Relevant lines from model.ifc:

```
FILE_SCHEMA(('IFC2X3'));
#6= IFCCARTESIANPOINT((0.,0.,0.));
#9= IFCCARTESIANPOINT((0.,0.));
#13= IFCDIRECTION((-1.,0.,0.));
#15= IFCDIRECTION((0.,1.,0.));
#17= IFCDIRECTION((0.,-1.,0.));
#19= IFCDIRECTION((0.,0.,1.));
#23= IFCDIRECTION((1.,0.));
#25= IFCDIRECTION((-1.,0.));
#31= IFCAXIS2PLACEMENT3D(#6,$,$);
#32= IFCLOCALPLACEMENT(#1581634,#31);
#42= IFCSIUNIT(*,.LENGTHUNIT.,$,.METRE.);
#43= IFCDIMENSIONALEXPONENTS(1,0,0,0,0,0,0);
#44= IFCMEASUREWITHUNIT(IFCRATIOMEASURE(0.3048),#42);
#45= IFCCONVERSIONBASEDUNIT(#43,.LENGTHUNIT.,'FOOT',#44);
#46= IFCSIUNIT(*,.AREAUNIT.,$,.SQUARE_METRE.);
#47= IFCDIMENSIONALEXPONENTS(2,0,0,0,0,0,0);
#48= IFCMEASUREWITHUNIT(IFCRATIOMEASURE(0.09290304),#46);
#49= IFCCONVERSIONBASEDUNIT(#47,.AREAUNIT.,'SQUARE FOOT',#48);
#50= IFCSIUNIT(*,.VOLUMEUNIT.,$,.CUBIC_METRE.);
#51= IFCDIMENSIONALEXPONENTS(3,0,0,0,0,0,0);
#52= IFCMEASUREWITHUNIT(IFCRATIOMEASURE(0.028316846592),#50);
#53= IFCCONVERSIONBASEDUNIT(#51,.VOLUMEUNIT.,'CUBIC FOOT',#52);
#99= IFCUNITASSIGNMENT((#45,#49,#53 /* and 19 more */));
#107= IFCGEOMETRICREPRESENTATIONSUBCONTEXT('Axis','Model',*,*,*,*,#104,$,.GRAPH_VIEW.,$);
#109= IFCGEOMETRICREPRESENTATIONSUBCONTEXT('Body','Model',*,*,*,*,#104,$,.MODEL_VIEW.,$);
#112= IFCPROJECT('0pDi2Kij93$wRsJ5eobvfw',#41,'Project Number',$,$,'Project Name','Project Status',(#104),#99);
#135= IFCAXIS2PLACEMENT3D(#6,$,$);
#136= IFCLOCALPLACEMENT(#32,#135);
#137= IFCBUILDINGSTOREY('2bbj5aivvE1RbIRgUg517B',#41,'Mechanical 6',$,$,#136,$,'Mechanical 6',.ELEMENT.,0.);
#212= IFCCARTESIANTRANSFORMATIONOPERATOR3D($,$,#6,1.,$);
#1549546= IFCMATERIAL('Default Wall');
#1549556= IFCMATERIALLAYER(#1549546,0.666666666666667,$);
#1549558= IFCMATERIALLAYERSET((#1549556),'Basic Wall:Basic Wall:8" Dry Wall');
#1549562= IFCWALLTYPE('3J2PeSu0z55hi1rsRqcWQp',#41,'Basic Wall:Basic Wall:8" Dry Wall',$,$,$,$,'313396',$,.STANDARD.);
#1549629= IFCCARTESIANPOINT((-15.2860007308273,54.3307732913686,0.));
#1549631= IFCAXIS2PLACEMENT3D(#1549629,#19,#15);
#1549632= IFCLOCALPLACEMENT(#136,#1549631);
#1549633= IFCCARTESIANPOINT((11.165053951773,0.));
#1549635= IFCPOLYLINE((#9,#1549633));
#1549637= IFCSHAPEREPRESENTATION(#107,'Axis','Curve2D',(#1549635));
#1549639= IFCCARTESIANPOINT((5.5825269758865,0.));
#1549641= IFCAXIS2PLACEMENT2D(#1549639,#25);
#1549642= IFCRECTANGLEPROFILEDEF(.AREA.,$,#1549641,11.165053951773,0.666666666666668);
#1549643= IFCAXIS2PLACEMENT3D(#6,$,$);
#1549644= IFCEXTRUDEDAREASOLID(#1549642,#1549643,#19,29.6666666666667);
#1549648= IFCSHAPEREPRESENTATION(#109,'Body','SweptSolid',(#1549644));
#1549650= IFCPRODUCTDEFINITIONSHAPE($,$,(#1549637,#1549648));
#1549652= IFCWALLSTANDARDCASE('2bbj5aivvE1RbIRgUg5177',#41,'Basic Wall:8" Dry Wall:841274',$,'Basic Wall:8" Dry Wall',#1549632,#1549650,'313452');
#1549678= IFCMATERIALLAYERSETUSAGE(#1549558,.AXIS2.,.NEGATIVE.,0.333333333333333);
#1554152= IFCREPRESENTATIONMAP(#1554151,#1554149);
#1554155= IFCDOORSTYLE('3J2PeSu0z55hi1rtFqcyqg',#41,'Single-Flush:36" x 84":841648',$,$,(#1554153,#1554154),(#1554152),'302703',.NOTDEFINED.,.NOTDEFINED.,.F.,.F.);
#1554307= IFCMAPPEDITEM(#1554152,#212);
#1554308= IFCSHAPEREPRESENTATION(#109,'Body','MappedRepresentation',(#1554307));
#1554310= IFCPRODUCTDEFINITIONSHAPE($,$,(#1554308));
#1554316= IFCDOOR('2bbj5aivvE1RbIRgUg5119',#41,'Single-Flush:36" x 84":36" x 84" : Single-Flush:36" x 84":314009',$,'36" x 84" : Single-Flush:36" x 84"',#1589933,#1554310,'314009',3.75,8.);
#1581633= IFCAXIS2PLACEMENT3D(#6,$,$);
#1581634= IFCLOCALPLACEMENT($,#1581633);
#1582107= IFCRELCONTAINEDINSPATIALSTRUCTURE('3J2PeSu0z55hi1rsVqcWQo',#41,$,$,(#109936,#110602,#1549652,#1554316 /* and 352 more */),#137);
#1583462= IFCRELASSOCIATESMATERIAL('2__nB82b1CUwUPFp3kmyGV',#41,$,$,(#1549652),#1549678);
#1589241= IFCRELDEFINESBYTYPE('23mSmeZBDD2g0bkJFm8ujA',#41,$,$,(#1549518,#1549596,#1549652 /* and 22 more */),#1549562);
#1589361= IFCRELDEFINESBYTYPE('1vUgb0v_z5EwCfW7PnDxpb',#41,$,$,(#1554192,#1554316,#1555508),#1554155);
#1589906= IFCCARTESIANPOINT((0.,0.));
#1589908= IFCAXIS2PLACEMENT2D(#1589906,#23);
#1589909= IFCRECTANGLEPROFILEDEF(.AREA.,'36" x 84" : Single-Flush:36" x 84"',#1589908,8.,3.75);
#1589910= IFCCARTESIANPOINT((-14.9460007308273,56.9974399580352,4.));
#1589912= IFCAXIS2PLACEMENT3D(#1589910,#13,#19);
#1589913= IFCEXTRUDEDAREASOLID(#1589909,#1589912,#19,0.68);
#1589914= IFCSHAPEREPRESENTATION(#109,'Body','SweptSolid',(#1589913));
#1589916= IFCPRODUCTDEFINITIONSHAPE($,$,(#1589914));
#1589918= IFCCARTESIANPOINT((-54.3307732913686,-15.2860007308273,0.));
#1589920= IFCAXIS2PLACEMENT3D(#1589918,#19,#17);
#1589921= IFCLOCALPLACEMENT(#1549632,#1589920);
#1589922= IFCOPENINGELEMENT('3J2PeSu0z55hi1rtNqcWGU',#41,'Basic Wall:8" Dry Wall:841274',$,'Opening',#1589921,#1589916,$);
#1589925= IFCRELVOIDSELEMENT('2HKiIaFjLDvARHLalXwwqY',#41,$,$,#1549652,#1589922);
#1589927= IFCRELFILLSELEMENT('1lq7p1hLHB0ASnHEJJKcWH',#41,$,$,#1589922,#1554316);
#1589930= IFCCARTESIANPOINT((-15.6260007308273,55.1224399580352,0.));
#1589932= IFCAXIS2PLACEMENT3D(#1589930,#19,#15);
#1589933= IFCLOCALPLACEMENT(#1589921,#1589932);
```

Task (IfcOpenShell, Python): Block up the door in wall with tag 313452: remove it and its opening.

```python
import ifcopenshell
import ifcopenshell.api.feature
import ifcopenshell.api.root
import ifcopenshell.geom
import ifcopenshell.util.shape

model = ifcopenshell.open("model.ifc")
settings = ifcopenshell.geom.settings()


def volume(element):
    """Net volume in cubic metres, openings subtracted."""
    shape = ifcopenshell.geom.create_shape(settings, element)
    return ifcopenshell.util.shape.get_volume(shape.geometry)


door = model.by_id(1554316)
opening = door.FillsVoids[0].RelatingOpeningElement
wall = opening.VoidsElements[0].RelatingBuildingElement
before = volume(wall)

ifcopenshell.api.root.remove_product(model, product=door)
ifcopenshell.api.feature.remove_feature(model, feature=opening)

after = volume(wall)

print(f"wall volume {before:.3f} -> {after:.3f} m3")

model.write("model_updated.ifc")
```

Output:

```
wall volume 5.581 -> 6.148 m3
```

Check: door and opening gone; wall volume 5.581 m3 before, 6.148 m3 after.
